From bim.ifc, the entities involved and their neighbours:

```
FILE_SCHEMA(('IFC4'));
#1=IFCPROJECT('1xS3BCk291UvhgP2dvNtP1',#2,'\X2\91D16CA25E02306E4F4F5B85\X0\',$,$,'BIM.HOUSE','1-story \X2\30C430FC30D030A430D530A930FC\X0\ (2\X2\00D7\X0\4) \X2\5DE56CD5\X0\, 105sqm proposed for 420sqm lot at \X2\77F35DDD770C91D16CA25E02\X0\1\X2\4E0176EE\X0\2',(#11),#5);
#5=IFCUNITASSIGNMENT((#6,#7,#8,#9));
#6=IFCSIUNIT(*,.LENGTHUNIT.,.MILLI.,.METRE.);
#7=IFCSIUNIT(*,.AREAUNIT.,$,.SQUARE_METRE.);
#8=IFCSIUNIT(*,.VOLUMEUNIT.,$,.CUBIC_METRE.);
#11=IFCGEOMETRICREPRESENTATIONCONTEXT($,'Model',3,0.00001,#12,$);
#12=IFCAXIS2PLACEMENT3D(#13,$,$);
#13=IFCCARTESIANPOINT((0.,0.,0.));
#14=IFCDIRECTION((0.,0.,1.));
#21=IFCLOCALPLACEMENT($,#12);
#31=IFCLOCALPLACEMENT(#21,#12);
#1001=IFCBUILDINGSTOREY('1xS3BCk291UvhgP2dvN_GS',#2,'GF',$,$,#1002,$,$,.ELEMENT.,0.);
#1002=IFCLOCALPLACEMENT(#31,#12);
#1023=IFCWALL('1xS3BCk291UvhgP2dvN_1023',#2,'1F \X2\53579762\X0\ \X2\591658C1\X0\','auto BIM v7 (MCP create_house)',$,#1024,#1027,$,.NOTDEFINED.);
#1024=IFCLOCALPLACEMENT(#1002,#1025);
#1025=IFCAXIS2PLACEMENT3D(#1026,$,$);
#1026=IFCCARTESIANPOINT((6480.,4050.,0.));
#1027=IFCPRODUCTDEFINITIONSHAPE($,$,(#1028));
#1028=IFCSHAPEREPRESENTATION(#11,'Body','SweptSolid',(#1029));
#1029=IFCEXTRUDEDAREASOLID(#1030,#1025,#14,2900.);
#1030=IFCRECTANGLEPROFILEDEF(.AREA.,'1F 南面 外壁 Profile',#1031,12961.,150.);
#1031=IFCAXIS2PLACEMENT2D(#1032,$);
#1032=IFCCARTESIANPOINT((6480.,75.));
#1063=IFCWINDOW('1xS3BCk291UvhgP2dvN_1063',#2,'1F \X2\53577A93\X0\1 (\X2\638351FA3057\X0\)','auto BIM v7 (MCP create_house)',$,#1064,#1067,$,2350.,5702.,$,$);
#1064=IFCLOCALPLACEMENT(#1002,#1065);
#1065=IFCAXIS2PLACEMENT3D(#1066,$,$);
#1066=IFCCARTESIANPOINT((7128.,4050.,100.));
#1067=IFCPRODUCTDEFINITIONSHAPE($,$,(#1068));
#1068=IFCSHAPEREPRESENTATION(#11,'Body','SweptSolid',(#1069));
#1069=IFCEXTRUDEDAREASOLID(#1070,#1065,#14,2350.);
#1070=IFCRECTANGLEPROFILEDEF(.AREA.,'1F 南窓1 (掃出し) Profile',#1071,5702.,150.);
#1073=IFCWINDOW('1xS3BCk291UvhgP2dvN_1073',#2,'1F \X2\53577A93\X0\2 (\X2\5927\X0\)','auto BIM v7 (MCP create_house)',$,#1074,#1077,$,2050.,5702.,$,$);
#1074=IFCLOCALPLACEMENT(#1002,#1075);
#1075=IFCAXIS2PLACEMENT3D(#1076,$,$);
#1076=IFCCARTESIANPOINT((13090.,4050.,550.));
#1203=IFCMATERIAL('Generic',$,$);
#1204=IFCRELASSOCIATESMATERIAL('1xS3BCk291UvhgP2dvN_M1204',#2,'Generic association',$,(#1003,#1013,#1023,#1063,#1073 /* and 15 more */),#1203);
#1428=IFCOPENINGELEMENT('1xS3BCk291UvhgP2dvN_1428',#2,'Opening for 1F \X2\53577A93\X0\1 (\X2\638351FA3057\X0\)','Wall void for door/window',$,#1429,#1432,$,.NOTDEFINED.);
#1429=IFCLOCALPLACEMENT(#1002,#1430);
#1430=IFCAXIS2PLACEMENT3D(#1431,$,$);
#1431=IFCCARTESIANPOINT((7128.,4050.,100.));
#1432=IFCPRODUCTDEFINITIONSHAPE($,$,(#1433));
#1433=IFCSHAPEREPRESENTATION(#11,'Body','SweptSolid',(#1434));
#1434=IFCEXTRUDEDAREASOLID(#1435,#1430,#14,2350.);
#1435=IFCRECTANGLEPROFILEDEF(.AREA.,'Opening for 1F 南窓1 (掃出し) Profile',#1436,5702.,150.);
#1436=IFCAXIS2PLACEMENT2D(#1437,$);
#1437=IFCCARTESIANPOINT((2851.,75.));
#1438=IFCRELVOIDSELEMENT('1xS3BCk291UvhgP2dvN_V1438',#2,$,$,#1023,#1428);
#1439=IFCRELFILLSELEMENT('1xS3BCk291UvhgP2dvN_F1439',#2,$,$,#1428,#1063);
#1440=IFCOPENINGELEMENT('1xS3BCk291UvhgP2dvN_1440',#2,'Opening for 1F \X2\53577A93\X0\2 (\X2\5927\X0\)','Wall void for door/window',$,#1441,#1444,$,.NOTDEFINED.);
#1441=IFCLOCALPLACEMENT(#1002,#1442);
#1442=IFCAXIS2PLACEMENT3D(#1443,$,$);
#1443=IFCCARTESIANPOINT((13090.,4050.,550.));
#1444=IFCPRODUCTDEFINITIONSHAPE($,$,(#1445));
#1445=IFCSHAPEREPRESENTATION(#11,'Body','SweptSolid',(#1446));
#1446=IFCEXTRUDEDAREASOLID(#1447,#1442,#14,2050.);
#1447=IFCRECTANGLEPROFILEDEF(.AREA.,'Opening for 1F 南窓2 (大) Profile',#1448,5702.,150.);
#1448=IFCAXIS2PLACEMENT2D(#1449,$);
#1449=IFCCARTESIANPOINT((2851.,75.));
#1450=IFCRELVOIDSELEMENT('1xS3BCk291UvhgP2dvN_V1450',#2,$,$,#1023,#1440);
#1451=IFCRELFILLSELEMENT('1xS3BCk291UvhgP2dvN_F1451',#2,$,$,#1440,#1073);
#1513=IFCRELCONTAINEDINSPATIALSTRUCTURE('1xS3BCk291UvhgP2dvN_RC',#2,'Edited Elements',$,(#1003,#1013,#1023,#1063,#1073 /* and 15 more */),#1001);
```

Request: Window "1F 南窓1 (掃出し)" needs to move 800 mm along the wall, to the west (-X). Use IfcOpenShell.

```python
import ifcopenshell
import ifcopenshell.api.geometry
import ifcopenshell.util.placement

model = ifcopenshell.open("bim.ifc")

window = model.by_guid("1xS3BCk291UvhgP2dvN_1063")
opening = window.FillsVoids[0].RelatingOpeningElement
wall = opening.VoidsElements[0].RelatingBuildingElement

wall_matrix = ifcopenshell.util.placement.get_local_placement(wall.ObjectPlacement)
shift = wall_matrix[:3, 0] * -800.0
before = ifcopenshell.util.placement.get_local_placement(window.ObjectPlacement)[:3, 3].copy()

# The window is not placed relative to its opening, so move both.
for product in (opening, window):
    matrix = ifcopenshell.util.placement.get_local_placement(product.ObjectPlacement)
    matrix[:3, 3] += shift
    ifcopenshell.api.geometry.edit_object_placement(model, product=product, matrix=matrix, is_si=False)

after = ifcopenshell.util.placement.get_local_placement(window.ObjectPlacement)[:3, 3]
print("window moved by", (after - before).round(3) + 0.0)

model.write("bim_edited.ifc")
```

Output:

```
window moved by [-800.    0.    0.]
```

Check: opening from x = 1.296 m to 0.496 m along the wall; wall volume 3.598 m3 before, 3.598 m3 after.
